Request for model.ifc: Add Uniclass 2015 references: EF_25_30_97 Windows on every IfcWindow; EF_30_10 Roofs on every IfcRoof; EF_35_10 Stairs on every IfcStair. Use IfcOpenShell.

First a look at what the model holds.

```python
import ifcopenshell

model = ifcopenshell.open("model.ifc")
print(model.schema)
print("classifications:", [c.Name for c in model.by_type("IfcClassification")])
for ifc_class in ("IfcDoor", "IfcRoof", "IfcStair", "IfcWall", "IfcWindow"):
    print(ifc_class, len(model.by_type(ifc_class)))
```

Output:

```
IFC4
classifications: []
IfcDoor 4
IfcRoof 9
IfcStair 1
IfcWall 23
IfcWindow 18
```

```python
import ifcopenshell
import ifcopenshell.api.classification

model = ifcopenshell.open("model.ifc")

system = ifcopenshell.api.classification.add_classification(model, classification="Uniclass 2015")

codes = {
    "IfcWindow": ("EF_25_30_97", "Windows"),
    "IfcRoof": ("EF_30_10", "Roofs"),
    "IfcStair": ("EF_35_10", "Stairs"),
}
for ifc_class, (code, name) in codes.items():
    products = model.by_type(ifc_class)
    ifcopenshell.api.classification.add_reference(
        model, products=products, classification=system, identification=code, name=name
    )
    print(code, len(products))

model.write("model_updated.ifc")
```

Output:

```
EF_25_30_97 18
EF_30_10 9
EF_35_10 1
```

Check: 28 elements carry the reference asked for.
